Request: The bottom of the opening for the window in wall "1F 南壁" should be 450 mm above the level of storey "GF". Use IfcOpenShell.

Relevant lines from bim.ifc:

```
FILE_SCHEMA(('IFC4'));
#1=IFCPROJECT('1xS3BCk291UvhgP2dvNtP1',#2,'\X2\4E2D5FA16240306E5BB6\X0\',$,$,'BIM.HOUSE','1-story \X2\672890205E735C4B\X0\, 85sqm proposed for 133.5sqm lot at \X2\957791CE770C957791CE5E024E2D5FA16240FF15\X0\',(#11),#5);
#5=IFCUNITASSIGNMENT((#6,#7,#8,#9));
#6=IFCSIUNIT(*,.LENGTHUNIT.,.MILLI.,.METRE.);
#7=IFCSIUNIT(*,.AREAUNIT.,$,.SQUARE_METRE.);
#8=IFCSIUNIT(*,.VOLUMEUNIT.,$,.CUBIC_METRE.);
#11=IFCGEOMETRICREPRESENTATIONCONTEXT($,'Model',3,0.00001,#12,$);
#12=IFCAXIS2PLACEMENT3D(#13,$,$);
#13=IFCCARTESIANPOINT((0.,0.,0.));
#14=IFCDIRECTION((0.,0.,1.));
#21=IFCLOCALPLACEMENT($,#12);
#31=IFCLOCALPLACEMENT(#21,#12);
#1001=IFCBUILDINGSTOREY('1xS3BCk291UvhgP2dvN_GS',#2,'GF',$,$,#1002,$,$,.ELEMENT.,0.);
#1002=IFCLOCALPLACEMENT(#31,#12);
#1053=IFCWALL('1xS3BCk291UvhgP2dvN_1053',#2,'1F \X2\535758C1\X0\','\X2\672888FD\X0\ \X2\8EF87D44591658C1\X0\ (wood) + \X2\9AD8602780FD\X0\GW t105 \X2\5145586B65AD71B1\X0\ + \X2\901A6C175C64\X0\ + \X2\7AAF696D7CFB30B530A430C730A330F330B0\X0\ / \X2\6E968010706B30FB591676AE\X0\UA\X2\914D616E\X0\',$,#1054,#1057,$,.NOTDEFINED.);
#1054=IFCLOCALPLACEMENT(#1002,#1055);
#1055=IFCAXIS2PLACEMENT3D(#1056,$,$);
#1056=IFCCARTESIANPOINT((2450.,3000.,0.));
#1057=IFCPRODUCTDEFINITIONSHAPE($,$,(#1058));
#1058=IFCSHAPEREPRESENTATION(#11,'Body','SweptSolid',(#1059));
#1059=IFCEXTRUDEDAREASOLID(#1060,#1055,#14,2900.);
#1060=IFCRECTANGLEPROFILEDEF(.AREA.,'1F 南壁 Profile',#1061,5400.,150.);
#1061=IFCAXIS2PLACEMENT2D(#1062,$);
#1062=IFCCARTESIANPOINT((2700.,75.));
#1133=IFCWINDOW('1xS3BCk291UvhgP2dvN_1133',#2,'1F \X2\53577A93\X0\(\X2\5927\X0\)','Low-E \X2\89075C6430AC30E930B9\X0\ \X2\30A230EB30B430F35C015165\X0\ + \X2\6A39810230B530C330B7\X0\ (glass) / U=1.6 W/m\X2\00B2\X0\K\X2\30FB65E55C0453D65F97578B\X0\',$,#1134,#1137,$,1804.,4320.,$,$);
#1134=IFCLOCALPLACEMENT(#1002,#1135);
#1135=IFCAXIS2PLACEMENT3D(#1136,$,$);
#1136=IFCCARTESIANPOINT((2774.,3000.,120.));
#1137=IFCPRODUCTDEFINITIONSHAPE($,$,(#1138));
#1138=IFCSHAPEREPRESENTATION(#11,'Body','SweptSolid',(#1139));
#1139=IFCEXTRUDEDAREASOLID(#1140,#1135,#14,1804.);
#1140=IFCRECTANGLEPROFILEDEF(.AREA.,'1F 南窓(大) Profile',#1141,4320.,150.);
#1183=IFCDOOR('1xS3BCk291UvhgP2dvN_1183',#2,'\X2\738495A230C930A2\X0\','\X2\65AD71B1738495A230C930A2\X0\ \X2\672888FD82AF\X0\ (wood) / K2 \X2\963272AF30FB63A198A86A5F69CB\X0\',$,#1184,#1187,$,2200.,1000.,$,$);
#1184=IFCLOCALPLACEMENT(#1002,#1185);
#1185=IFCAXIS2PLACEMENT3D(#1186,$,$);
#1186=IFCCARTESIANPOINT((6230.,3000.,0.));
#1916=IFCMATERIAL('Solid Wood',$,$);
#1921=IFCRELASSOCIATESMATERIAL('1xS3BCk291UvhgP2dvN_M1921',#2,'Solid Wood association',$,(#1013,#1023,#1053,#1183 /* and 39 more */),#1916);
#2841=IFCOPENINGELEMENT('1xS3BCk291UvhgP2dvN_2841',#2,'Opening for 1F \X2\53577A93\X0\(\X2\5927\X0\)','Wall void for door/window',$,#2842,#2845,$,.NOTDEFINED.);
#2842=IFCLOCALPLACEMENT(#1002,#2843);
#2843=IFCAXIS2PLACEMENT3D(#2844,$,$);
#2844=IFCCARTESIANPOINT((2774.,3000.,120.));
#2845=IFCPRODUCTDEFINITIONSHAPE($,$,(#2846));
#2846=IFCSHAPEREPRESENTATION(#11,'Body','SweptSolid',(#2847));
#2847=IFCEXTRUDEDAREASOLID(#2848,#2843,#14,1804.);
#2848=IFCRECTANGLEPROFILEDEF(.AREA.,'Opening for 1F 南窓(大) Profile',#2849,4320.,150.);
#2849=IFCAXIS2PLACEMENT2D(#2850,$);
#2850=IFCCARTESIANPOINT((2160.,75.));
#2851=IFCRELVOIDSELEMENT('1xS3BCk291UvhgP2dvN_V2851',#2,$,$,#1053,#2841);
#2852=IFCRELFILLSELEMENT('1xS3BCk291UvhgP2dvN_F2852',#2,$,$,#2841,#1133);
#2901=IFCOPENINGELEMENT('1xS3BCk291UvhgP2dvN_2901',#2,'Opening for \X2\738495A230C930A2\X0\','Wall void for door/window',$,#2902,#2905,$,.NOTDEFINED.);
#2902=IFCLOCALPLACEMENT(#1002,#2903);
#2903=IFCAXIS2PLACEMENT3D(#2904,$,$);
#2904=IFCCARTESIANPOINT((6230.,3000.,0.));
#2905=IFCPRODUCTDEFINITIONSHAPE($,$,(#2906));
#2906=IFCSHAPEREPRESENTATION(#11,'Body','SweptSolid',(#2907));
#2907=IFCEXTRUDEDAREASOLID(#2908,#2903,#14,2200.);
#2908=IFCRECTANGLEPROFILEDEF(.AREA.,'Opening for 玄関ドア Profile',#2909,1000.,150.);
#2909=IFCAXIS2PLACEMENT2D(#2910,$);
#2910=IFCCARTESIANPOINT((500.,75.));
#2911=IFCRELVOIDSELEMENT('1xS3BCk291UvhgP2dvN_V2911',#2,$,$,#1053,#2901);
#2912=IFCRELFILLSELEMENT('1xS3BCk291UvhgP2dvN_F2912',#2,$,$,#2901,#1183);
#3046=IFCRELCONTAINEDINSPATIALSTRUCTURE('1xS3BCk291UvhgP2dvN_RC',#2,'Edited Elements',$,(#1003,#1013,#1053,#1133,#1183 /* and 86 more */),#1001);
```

```python
import numpy as np
import ifcopenshell
import ifcopenshell.api.geometry
import ifcopenshell.geom
import ifcopenshell.util.element
import ifcopenshell.util.placement
import ifcopenshell.util.shape
import ifcopenshell.util.unit

model = ifcopenshell.open("bim.ifc")
unit_scale = ifcopenshell.util.unit.calculate_unit_scale(model)

window = model.by_guid("1xS3BCk291UvhgP2dvN_1133")
opening = window.FillsVoids[0].RelatingOpeningElement
storey = ifcopenshell.util.element.get_container(window, ifc_class="IfcBuildingStorey")
level = ifcopenshell.util.placement.get_local_placement(storey.ObjectPlacement)[2, 3]

# The opening's origin need not be at the sill, so measure its lowest point.
shape = ifcopenshell.geom.create_shape(ifcopenshell.geom.settings(), opening)
bottom = ifcopenshell.util.shape.get_shape_bottom_elevation(shape, shape.geometry) / unit_scale
dz = level + 450.0 - bottom

shift = np.array([0.0, 0.0, dz])
# The window is not placed relative to its opening, so move both.
for product in (opening, window):
    matrix = ifcopenshell.util.placement.get_local_placement(product.ObjectPlacement)
    matrix[:3, 3] += shift
    ifcopenshell.api.geometry.edit_object_placement(model, product=product, matrix=matrix, is_si=False)

print(f"moved by {dz * unit_scale:+.3f} m")

model.write("bim_updated.ifc")
```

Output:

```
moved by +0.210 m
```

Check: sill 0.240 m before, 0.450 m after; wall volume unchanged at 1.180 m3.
